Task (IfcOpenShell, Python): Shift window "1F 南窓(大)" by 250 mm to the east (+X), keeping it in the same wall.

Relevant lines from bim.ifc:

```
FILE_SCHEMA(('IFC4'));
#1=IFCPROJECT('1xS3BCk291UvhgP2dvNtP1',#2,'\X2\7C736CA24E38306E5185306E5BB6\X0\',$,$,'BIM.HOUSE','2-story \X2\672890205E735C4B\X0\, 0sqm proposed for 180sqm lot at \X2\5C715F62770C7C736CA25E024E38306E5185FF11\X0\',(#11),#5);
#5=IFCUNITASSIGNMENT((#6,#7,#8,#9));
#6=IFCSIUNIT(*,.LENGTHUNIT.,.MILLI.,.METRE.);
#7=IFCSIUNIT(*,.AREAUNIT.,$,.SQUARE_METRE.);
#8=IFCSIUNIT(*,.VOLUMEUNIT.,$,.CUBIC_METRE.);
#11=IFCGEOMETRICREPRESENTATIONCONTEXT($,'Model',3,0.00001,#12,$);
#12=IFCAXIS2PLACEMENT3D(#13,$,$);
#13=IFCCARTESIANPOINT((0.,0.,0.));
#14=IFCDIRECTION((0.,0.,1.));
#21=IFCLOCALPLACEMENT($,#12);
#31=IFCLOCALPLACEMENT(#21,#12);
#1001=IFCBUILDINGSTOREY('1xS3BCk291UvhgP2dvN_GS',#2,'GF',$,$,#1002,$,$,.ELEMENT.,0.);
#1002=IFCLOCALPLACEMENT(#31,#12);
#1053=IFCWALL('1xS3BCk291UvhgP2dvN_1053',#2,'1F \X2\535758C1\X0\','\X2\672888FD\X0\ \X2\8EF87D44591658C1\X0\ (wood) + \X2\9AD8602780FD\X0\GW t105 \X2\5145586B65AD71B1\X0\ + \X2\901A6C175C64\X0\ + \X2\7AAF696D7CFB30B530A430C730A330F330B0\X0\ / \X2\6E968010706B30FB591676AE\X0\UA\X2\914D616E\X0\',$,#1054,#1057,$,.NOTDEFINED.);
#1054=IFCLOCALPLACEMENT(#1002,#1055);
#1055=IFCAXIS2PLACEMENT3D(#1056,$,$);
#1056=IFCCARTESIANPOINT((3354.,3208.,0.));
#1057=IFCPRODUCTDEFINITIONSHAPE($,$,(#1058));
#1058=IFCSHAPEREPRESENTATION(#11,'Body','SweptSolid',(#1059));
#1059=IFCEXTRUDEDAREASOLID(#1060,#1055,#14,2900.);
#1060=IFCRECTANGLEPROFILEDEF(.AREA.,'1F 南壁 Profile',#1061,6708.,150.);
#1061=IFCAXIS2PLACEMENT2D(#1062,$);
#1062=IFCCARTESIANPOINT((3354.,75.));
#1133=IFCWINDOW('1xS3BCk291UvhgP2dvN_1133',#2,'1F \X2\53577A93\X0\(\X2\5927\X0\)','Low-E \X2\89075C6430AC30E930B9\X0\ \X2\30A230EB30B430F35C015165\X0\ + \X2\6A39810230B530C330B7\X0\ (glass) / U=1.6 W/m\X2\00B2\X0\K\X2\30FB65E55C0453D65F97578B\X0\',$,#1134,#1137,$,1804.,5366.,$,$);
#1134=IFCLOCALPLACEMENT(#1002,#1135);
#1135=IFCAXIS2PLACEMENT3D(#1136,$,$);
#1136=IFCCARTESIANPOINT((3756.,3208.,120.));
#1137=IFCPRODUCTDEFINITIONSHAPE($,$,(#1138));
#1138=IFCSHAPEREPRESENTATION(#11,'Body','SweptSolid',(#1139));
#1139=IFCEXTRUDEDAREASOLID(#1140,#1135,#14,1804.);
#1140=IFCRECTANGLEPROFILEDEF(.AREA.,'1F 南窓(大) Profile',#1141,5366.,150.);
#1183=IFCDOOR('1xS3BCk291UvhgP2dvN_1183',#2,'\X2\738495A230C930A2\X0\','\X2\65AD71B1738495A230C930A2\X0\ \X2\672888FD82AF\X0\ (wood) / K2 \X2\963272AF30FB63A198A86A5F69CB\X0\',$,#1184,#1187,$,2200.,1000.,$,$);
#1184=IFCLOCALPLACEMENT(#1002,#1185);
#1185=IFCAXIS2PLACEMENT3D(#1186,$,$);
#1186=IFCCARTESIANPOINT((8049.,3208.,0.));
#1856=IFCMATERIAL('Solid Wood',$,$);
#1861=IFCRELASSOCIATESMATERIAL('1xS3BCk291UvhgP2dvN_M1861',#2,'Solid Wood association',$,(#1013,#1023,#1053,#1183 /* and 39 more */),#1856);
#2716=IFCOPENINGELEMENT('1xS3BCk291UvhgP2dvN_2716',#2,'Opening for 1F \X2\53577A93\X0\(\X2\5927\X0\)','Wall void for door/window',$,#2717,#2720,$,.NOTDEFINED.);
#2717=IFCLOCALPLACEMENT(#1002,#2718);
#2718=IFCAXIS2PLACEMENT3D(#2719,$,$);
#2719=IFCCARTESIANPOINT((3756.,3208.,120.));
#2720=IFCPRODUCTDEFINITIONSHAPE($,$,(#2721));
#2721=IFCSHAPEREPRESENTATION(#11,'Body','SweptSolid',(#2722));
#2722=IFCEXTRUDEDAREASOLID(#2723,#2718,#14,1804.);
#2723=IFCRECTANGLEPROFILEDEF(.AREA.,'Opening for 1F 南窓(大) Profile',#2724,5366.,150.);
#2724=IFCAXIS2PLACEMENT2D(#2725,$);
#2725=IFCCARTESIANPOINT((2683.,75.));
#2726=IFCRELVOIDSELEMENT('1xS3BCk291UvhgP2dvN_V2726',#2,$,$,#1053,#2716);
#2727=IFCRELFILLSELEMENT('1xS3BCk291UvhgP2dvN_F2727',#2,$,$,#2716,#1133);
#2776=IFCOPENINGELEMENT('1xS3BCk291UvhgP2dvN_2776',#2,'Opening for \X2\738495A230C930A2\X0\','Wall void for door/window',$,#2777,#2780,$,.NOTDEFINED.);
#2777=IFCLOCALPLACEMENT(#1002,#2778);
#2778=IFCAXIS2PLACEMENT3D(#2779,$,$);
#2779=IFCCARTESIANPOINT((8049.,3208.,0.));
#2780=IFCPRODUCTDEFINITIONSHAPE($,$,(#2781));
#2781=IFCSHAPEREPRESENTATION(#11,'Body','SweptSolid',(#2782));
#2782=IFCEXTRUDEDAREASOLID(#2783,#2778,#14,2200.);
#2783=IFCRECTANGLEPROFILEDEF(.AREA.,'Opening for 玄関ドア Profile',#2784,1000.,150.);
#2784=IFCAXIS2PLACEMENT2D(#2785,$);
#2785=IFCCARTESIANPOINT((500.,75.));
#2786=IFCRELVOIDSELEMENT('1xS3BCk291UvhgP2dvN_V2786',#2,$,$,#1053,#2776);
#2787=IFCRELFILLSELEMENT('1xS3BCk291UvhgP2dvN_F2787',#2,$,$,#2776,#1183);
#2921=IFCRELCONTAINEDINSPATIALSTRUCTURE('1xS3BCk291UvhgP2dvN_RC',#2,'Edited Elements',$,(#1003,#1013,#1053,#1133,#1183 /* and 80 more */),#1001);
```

```python
import ifcopenshell
import ifcopenshell.api.geometry
import ifcopenshell.util.placement
import ifcopenshell.util.unit

model = ifcopenshell.open("bim.ifc")
unit_scale = ifcopenshell.util.unit.calculate_unit_scale(model)

window = model.by_guid("1xS3BCk291UvhgP2dvN_1133")
opening = window.FillsVoids[0].RelatingOpeningElement
wall = opening.VoidsElements[0].RelatingBuildingElement

wall_matrix = ifcopenshell.util.placement.get_local_placement(wall.ObjectPlacement)
shift = wall_matrix[:3, 0] * 0.25 / unit_scale
before = ifcopenshell.util.placement.get_local_placement(window.ObjectPlacement)[:3, 3].copy()

# The window is not placed relative to its opening, so move both.
for product in (opening, window):
    matrix = ifcopenshell.util.placement.get_local_placement(product.ObjectPlacement)
    matrix[:3, 3] += shift
    ifcopenshell.api.geometry.edit_object_placement(model, product=product, matrix=matrix, is_si=False)

after = ifcopenshell.util.placement.get_local_placement(window.ObjectPlacement)[:3, 3]
print("window moved by", (after - before).round(3) + 0.0)

model.write("bim_rev.ifc")
```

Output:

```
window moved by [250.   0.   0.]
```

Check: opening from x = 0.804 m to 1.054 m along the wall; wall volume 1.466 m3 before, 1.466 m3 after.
